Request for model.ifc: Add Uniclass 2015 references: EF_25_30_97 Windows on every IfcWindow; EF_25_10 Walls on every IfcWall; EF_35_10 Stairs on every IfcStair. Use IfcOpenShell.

First a look at what the model holds.

```python
import ifcopenshell

model = ifcopenshell.open("model.ifc")
print(model.schema)
print("classifications:", [c.Name for c in model.by_type("IfcClassification")])
for ifc_class in ("IfcDoor", "IfcRoof", "IfcStair", "IfcWall", "IfcWindow"):
    print(ifc_class, len(model.by_type(ifc_class)))
```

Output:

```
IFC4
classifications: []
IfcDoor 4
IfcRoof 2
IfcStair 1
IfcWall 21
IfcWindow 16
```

```python
import ifcopenshell
import ifcopenshell.api.classification

model = ifcopenshell.open("model.ifc")

system = ifcopenshell.api.classification.add_classification(model, classification="Uniclass 2015")

codes = {
    "IfcWindow": ("EF_25_30_97", "Windows"),
    "IfcWall": ("EF_25_10", "Walls"),
    "IfcStair": ("EF_35_10", "Stairs"),
}
for ifc_class, (code, name) in codes.items():
    products = model.by_type(ifc_class)
    ifcopenshell.api.classification.add_reference(
        model, products=products, classification=system, identification=code, name=name
    )
    print(code, len(products))

model.write("model_updated.ifc")
```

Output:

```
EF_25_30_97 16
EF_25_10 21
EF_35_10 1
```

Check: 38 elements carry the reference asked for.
